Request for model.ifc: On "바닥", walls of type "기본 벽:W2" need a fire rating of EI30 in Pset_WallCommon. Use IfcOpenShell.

First a look at what the model holds.

```python
import ifcopenshell
import ifcopenshell.util.element

model = ifcopenshell.open("model.ifc")
print(model.schema)
storey = next(s for s in model.by_type("IfcBuildingStorey") if s.Name == "바닥")
walls = [e for e in ifcopenshell.util.element.get_decomposition(storey) if e.is_a("IfcWall")]
seen = {}
for e in walls:
    element_type = ifcopenshell.util.element.get_type(e)
    key = (element_type.Name if element_type != e and element_type else None, ifcopenshell.util.element.get_pset(e, "Pset_WallCommon", "FireRating"))
    seen[key] = seen.get(key, 0) + 1
for (name, value), count in sorted(seen.items(), key=str):
    print(count, "x", name, "|", value)
```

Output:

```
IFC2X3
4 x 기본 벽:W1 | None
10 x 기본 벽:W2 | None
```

```python
import ifcopenshell
import ifcopenshell.api.pset
import ifcopenshell.util.element

model = ifcopenshell.open("model.ifc")

storey = next(s for s in model.by_type("IfcBuildingStorey") if s.Name == "바닥")
walls = [e for e in ifcopenshell.util.element.get_decomposition(storey) if e.is_a("IfcWall")]

count = 0
for e in walls:
    element_type = ifcopenshell.util.element.get_type(e)
    if element_type in (None, e) or element_type.Name != "기본 벽:W2":
        continue
    # add_pset returns the element's existing set when there is one.
    pset = ifcopenshell.api.pset.add_pset(model, product=e, name="Pset_WallCommon")
    ifcopenshell.api.pset.edit_pset(model, pset=pset, properties={"FireRating": "EI30"})
    count += 1

print(count, "walls updated")

model.write("model_updated.ifc")
```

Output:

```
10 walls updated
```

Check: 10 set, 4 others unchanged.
